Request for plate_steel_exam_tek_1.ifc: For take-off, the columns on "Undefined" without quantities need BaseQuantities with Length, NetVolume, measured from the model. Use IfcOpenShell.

First a look at what the model holds.

```python
import ifcopenshell
import ifcopenshell.util.element
import ifcopenshell.util.unit

model = ifcopenshell.open("plate_steel_exam_tek_1.ifc")
print(model.schema)
for unit_type in ("LENGTHUNIT", "AREAUNIT", "VOLUMEUNIT"):
    print(unit_type, ifcopenshell.util.unit.calculate_unit_scale(model, unit_type))
storey = next(s for s in model.by_type("IfcBuildingStorey") if s.Name == "Undefined")
columns = [e for e in ifcopenshell.util.element.get_decomposition(storey) if e.is_a("IfcColumn")]
for e in sorted(columns, key=lambda e: e.id()):
    print(e.id(), e.is_a(), e.Name, list(ifcopenshell.util.element.get_psets(e, qtos_only=True)), sep=" | ")
```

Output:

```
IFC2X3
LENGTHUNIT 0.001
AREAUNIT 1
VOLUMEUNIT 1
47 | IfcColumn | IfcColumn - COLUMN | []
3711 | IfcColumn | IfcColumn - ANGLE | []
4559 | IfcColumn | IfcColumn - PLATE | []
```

```python
import ifcopenshell
import ifcopenshell.api.pset
import ifcopenshell.geom
import ifcopenshell.util.element
import ifcopenshell.util.shape
import ifcopenshell.util.unit

model = ifcopenshell.open("plate_steel_exam_tek_1.ifc")
unit_scale = ifcopenshell.util.unit.calculate_unit_scale(model)
volume_scale = ifcopenshell.util.unit.calculate_unit_scale(model, "VOLUMEUNIT")
settings = ifcopenshell.geom.settings()

storey = next(s for s in model.by_type("IfcBuildingStorey") if s.Name == "Undefined")
columns = [e for e in ifcopenshell.util.element.get_decomposition(storey) if e.is_a("IfcColumn")]

for e in sorted(columns, key=lambda e: e.id()):
    if ifcopenshell.util.element.get_psets(e, qtos_only=True, should_inherit=False):
        continue
    # Geometry comes back in metres, in the element's own axes.
    shape = ifcopenshell.geom.create_shape(settings, e)
    values = {
        "Length": ifcopenshell.util.shape.get_z(shape.geometry) / unit_scale,
        "NetVolume": ifcopenshell.util.shape.get_volume(shape.geometry) / volume_scale,
    }
    qto = ifcopenshell.api.pset.add_qto(model, product=e, name="BaseQuantities")
    ifcopenshell.api.pset.edit_qto(model, qto=qto, properties=values)
    print(e.id(), {k: round(v, 3) for k, v in values.items()})

model.write("plate_steel_exam_tek_1-out.ifc")
```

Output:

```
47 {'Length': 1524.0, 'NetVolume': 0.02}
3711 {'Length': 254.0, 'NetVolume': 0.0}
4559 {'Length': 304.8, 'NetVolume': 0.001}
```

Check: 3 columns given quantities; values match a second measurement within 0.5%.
